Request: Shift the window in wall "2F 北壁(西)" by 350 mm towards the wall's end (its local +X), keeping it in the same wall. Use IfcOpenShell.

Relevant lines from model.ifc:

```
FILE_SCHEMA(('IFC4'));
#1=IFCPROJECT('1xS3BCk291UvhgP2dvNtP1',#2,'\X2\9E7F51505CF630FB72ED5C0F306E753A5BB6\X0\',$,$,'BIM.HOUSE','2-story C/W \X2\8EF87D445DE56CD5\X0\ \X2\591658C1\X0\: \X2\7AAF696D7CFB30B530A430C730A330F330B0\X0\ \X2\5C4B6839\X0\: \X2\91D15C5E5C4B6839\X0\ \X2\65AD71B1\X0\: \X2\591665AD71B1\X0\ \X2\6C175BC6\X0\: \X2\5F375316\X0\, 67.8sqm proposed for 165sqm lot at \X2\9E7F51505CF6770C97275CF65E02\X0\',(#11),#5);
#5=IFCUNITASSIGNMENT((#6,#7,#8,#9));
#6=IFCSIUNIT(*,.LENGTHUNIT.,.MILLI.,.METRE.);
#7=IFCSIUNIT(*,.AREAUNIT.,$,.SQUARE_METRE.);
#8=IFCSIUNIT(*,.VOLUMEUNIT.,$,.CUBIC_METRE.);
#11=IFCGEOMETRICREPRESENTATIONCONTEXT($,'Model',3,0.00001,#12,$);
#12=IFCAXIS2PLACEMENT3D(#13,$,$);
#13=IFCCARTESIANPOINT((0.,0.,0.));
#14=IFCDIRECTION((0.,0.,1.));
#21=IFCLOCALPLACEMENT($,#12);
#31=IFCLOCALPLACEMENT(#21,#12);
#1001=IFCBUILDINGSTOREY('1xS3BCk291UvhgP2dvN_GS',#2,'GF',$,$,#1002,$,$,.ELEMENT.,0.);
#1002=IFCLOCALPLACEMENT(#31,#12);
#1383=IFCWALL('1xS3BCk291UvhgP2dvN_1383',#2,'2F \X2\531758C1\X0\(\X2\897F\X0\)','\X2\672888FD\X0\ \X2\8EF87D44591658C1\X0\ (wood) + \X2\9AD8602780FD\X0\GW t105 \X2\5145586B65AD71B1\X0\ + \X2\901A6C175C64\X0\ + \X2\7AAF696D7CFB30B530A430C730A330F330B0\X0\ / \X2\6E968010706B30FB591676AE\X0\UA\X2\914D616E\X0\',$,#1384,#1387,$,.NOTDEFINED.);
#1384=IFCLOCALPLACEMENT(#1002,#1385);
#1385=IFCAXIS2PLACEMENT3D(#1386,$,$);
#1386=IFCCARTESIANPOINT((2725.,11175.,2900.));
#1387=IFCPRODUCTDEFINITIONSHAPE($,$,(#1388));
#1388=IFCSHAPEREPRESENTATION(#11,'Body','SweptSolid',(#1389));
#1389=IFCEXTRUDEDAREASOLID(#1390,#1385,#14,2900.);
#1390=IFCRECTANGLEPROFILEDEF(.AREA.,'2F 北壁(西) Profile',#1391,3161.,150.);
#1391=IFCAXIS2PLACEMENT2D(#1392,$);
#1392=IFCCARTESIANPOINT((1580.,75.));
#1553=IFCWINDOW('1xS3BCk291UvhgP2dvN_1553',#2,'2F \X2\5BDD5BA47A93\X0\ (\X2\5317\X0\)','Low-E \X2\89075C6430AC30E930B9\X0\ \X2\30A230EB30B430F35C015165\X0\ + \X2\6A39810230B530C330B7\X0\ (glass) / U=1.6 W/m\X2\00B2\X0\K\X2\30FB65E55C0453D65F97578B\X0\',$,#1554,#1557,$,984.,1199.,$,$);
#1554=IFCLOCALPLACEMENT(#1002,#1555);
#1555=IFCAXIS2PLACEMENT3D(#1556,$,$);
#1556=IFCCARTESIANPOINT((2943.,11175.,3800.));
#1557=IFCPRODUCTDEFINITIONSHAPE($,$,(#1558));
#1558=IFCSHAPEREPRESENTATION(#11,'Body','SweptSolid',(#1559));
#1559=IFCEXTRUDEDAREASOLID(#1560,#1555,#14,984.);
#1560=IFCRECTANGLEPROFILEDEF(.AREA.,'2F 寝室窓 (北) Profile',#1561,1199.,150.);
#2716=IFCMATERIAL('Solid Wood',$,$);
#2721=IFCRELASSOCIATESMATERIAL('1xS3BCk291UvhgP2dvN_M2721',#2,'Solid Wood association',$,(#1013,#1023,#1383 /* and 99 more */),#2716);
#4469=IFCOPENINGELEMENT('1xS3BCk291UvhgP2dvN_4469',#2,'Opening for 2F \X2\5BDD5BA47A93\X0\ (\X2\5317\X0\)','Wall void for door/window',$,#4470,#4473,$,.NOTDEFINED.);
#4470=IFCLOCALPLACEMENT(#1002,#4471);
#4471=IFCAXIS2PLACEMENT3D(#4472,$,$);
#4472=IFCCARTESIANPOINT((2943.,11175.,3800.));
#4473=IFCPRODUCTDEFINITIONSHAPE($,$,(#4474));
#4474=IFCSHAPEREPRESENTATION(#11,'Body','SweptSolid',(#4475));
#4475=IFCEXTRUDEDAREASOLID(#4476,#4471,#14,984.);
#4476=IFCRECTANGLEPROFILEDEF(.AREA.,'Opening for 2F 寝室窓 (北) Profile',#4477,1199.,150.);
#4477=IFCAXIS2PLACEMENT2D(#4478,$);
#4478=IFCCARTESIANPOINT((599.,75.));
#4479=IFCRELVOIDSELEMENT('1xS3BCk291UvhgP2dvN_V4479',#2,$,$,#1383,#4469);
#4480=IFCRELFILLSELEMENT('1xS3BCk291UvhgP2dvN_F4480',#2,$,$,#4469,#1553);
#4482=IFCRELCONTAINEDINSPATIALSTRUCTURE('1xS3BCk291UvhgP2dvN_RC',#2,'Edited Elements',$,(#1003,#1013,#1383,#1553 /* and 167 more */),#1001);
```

```python
import ifcopenshell
import ifcopenshell.api.geometry
import ifcopenshell.util.placement

model = ifcopenshell.open("model.ifc")

window = model.by_guid("1xS3BCk291UvhgP2dvN_1553")
opening = window.FillsVoids[0].RelatingOpeningElement
wall = opening.VoidsElements[0].RelatingBuildingElement

wall_matrix = ifcopenshell.util.placement.get_local_placement(wall.ObjectPlacement)
shift = wall_matrix[:3, 0] * 350.0
before = ifcopenshell.util.placement.get_local_placement(window.ObjectPlacement)[:3, 3].copy()

# The window is not placed relative to its opening, so move both.
for product in (opening, window):
    matrix = ifcopenshell.util.placement.get_local_placement(product.ObjectPlacement)
    matrix[:3, 3] += shift
    ifcopenshell.api.geometry.edit_object_placement(model, product=product, matrix=matrix, is_si=False)

after = ifcopenshell.util.placement.get_local_placement(window.ObjectPlacement)[:3, 3]
print("window moved by", (after - before).round(3) + 0.0)

model.write("model_rev.ifc")
```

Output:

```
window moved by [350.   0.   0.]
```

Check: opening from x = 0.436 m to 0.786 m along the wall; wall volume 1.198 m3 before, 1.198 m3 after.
